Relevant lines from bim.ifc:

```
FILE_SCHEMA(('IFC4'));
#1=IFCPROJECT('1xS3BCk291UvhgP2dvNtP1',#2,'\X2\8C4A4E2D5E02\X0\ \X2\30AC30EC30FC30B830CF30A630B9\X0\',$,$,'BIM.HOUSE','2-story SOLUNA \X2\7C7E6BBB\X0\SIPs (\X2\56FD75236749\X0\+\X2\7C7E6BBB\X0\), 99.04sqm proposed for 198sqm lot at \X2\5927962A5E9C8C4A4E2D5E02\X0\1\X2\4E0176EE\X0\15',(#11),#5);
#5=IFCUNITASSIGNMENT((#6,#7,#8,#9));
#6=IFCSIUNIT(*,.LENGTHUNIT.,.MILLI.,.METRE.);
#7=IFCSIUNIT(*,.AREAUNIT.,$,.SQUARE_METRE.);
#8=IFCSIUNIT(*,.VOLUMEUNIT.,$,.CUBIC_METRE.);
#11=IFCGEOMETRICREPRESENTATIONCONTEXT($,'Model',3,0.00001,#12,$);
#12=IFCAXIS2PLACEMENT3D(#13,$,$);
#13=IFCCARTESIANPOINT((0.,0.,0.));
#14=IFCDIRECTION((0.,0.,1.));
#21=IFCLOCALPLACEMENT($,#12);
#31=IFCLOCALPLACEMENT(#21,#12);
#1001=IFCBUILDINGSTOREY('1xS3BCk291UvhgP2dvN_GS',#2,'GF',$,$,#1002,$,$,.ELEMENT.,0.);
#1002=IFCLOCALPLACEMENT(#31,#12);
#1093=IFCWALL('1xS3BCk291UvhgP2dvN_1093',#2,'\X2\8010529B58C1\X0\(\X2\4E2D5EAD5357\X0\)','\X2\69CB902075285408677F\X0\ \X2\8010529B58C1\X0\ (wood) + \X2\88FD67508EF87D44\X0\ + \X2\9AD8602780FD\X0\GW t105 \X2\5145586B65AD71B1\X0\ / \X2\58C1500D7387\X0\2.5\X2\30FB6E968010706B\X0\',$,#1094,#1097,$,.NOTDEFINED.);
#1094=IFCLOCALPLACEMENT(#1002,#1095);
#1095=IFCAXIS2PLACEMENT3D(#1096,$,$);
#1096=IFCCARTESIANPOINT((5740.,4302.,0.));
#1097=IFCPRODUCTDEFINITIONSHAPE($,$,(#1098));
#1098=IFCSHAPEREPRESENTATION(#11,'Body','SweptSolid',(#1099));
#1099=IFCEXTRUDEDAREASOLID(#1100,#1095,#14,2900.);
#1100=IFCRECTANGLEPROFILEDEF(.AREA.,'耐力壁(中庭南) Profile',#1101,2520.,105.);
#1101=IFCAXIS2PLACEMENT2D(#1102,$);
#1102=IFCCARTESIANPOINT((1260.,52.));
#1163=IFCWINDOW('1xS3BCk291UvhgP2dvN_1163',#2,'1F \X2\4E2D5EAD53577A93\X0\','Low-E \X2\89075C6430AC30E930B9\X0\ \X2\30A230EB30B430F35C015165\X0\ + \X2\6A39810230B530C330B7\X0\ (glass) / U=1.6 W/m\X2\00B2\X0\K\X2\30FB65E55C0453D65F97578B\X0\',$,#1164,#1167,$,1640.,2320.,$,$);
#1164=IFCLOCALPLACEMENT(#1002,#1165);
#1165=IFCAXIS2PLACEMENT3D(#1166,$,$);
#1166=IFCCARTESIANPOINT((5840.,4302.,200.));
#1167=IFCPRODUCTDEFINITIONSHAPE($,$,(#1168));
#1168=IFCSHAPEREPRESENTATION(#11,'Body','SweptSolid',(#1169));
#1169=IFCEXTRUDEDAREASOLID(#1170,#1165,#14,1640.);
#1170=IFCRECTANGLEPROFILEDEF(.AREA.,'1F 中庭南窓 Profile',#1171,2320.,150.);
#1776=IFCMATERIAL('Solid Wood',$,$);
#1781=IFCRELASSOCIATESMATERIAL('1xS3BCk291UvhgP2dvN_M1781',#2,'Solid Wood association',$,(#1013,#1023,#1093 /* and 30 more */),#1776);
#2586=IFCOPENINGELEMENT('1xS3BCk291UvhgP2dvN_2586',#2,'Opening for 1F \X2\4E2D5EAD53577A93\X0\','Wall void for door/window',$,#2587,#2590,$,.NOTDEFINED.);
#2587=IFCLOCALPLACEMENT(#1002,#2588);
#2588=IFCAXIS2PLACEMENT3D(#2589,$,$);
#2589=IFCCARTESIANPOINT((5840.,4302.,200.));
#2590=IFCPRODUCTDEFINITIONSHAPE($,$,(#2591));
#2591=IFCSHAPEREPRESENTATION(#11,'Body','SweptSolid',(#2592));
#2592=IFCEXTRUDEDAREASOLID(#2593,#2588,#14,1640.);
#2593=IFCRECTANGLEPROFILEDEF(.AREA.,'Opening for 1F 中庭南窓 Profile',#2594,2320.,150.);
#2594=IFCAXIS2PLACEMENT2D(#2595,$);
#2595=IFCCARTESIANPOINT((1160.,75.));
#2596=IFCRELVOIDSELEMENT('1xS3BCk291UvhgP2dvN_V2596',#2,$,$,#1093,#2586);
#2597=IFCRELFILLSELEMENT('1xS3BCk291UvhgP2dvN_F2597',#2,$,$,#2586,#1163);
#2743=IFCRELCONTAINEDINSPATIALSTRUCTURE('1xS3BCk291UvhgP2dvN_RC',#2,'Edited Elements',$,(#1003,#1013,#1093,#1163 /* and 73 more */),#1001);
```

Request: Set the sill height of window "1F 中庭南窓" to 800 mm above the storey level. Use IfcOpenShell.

```python
import numpy as np
import ifcopenshell
import ifcopenshell.api.geometry
import ifcopenshell.geom
import ifcopenshell.util.element
import ifcopenshell.util.placement
import ifcopenshell.util.shape
import ifcopenshell.util.unit

model = ifcopenshell.open("bim.ifc")
unit_scale = ifcopenshell.util.unit.calculate_unit_scale(model)

window = model.by_id(1163)
opening = window.FillsVoids[0].RelatingOpeningElement
storey = ifcopenshell.util.element.get_container(window, ifc_class="IfcBuildingStorey")
level = ifcopenshell.util.placement.get_local_placement(storey.ObjectPlacement)[2, 3]

# The opening's origin need not be at the sill, so measure its lowest point.
shape = ifcopenshell.geom.create_shape(ifcopenshell.geom.settings(), opening)
bottom = ifcopenshell.util.shape.get_shape_bottom_elevation(shape, shape.geometry) / unit_scale
dz = level + 0.8 / unit_scale - bottom

shift = np.array([0.0, 0.0, dz])
# The window is not placed relative to its opening, so move both.
for product in (opening, window):
    matrix = ifcopenshell.util.placement.get_local_placement(product.ObjectPlacement)
    matrix[:3, 3] += shift
    ifcopenshell.api.geometry.edit_object_placement(model, product=product, matrix=matrix, is_si=False)

print(f"moved by {dz * unit_scale:+.3f} m")

model.write("bim-out.ifc")
```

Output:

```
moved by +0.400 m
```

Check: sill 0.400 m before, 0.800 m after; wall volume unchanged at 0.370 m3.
